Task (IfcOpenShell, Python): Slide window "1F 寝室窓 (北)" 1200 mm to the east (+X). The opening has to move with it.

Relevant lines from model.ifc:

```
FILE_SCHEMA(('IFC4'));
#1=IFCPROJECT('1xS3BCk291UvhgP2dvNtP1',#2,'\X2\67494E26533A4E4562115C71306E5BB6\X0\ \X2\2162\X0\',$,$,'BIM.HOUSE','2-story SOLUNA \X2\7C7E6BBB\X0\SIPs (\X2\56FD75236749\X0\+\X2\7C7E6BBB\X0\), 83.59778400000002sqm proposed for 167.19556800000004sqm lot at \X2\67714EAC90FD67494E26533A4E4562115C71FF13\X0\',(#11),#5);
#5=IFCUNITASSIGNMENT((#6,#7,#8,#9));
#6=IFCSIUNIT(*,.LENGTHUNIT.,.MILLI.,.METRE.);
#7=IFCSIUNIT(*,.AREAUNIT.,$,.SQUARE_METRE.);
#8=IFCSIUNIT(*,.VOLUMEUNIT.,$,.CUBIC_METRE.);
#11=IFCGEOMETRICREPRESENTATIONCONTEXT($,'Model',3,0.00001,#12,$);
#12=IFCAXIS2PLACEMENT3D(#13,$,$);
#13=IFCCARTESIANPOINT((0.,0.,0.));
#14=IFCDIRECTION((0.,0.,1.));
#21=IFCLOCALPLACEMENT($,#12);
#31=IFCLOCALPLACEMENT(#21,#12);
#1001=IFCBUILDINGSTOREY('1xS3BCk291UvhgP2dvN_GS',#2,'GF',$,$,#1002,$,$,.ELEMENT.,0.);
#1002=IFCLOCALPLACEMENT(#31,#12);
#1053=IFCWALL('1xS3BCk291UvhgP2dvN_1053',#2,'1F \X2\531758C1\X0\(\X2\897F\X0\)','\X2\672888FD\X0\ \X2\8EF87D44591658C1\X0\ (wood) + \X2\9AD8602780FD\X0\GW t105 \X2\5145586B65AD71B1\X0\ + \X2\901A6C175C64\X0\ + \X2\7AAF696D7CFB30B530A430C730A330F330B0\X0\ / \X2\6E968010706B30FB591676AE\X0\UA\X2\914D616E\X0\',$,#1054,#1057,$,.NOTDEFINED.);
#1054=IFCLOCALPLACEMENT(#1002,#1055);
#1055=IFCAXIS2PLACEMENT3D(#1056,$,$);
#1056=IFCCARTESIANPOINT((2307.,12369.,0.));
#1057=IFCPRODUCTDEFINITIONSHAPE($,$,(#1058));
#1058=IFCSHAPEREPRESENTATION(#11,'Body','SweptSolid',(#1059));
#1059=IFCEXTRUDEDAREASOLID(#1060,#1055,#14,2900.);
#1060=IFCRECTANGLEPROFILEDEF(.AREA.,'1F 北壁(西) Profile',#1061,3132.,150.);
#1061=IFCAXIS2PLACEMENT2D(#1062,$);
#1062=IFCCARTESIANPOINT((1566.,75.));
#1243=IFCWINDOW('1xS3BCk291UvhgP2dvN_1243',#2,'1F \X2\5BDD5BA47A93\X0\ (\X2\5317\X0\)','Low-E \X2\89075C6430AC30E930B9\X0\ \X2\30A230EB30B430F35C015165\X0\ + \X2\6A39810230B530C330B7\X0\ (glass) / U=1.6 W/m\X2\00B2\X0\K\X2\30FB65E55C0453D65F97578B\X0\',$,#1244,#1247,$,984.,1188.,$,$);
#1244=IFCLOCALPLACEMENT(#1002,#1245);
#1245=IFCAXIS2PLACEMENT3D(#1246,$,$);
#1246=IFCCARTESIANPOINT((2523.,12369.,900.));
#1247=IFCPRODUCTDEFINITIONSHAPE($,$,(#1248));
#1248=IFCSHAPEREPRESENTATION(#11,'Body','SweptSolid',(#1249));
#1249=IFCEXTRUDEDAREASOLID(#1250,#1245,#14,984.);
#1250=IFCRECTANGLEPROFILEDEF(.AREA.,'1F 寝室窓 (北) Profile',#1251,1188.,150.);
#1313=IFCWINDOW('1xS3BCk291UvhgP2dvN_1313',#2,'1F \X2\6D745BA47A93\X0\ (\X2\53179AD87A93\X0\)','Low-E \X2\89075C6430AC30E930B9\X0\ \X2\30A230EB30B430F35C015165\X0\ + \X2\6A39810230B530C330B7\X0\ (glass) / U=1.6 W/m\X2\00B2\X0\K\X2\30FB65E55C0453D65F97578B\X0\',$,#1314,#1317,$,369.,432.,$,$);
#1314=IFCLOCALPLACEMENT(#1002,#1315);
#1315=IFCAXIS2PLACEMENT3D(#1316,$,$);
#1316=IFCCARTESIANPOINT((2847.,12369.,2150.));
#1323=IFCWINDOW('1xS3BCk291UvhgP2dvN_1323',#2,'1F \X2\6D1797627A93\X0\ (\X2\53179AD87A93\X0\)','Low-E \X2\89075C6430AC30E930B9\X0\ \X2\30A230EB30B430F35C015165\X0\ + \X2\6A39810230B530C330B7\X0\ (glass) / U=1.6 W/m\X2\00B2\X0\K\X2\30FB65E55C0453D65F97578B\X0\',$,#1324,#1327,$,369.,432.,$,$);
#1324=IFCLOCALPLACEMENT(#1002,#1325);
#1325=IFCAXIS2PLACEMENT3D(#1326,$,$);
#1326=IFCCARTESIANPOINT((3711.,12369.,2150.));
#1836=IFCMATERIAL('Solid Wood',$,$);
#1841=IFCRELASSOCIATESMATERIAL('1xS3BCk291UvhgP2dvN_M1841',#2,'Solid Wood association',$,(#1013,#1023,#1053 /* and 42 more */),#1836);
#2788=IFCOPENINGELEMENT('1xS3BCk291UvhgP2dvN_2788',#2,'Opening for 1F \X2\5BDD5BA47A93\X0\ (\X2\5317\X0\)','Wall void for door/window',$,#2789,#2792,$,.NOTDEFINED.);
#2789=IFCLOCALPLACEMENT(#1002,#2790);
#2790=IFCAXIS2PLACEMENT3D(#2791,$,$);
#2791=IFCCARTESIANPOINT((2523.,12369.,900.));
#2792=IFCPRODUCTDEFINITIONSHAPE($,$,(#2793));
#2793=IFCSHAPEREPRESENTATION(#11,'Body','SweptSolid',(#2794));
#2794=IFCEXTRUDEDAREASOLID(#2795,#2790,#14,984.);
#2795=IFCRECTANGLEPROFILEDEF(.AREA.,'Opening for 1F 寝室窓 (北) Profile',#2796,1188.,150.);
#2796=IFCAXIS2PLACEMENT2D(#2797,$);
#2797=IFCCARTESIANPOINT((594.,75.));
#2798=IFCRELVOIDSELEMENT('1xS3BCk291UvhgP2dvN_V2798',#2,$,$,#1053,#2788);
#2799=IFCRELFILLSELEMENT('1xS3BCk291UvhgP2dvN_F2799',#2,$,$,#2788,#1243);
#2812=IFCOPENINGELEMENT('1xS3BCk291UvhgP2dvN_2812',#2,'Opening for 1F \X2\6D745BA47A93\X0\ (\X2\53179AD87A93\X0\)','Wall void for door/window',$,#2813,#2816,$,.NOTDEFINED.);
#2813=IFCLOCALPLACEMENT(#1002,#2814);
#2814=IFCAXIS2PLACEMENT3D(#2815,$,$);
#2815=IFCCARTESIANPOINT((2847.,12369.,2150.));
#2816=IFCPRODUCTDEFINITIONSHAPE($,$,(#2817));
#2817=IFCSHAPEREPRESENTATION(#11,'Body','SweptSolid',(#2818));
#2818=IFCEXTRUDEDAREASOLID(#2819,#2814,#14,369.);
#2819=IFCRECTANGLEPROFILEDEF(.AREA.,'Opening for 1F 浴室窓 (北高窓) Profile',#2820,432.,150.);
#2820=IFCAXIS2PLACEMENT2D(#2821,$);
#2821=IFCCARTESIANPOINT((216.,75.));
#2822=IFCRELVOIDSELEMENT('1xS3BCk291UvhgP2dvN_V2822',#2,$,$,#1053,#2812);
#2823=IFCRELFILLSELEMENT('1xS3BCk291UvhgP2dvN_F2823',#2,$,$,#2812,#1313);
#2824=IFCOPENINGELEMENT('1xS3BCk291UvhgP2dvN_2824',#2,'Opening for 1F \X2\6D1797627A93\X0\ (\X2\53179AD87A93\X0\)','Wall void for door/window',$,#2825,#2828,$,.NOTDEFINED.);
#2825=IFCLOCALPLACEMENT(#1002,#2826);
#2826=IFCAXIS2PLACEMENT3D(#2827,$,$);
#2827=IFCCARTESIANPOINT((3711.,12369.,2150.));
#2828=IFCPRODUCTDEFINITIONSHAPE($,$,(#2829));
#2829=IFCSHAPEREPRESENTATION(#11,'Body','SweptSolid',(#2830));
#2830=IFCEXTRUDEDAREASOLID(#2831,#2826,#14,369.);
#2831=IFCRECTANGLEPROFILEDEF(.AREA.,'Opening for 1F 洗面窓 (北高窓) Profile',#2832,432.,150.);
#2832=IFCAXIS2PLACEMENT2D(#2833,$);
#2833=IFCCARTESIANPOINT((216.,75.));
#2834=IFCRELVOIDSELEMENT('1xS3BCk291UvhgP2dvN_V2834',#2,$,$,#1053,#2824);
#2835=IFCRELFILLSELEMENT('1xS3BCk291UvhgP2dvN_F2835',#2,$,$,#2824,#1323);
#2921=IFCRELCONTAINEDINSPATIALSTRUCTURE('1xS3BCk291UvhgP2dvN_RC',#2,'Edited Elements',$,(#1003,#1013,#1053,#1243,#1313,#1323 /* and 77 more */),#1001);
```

```python
import ifcopenshell
import ifcopenshell.api.geometry
import ifcopenshell.util.placement
import ifcopenshell.util.unit

model = ifcopenshell.open("model.ifc")
unit_scale = ifcopenshell.util.unit.calculate_unit_scale(model)

window = model.by_guid("1xS3BCk291UvhgP2dvN_1243")
opening = window.FillsVoids[0].RelatingOpeningElement
wall = opening.VoidsElements[0].RelatingBuildingElement

wall_matrix = ifcopenshell.util.placement.get_local_placement(wall.ObjectPlacement)
shift = wall_matrix[:3, 0] * 1.2 / unit_scale
before = ifcopenshell.util.placement.get_local_placement(window.ObjectPlacement)[:3, 3].copy()

# The window is not placed relative to its opening, so move both.
for product in (opening, window):
    matrix = ifcopenshell.util.placement.get_local_placement(product.ObjectPlacement)
    matrix[:3, 3] += shift
    ifcopenshell.api.geometry.edit_object_placement(model, product=product, matrix=matrix, is_si=False)

after = ifcopenshell.util.placement.get_local_placement(window.ObjectPlacement)[:3, 3]
print("window moved by", (after - before).round(3) + 0.0)

model.write("model_rev.ifc")
```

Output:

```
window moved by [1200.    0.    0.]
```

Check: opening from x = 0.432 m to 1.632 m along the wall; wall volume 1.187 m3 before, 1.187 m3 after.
